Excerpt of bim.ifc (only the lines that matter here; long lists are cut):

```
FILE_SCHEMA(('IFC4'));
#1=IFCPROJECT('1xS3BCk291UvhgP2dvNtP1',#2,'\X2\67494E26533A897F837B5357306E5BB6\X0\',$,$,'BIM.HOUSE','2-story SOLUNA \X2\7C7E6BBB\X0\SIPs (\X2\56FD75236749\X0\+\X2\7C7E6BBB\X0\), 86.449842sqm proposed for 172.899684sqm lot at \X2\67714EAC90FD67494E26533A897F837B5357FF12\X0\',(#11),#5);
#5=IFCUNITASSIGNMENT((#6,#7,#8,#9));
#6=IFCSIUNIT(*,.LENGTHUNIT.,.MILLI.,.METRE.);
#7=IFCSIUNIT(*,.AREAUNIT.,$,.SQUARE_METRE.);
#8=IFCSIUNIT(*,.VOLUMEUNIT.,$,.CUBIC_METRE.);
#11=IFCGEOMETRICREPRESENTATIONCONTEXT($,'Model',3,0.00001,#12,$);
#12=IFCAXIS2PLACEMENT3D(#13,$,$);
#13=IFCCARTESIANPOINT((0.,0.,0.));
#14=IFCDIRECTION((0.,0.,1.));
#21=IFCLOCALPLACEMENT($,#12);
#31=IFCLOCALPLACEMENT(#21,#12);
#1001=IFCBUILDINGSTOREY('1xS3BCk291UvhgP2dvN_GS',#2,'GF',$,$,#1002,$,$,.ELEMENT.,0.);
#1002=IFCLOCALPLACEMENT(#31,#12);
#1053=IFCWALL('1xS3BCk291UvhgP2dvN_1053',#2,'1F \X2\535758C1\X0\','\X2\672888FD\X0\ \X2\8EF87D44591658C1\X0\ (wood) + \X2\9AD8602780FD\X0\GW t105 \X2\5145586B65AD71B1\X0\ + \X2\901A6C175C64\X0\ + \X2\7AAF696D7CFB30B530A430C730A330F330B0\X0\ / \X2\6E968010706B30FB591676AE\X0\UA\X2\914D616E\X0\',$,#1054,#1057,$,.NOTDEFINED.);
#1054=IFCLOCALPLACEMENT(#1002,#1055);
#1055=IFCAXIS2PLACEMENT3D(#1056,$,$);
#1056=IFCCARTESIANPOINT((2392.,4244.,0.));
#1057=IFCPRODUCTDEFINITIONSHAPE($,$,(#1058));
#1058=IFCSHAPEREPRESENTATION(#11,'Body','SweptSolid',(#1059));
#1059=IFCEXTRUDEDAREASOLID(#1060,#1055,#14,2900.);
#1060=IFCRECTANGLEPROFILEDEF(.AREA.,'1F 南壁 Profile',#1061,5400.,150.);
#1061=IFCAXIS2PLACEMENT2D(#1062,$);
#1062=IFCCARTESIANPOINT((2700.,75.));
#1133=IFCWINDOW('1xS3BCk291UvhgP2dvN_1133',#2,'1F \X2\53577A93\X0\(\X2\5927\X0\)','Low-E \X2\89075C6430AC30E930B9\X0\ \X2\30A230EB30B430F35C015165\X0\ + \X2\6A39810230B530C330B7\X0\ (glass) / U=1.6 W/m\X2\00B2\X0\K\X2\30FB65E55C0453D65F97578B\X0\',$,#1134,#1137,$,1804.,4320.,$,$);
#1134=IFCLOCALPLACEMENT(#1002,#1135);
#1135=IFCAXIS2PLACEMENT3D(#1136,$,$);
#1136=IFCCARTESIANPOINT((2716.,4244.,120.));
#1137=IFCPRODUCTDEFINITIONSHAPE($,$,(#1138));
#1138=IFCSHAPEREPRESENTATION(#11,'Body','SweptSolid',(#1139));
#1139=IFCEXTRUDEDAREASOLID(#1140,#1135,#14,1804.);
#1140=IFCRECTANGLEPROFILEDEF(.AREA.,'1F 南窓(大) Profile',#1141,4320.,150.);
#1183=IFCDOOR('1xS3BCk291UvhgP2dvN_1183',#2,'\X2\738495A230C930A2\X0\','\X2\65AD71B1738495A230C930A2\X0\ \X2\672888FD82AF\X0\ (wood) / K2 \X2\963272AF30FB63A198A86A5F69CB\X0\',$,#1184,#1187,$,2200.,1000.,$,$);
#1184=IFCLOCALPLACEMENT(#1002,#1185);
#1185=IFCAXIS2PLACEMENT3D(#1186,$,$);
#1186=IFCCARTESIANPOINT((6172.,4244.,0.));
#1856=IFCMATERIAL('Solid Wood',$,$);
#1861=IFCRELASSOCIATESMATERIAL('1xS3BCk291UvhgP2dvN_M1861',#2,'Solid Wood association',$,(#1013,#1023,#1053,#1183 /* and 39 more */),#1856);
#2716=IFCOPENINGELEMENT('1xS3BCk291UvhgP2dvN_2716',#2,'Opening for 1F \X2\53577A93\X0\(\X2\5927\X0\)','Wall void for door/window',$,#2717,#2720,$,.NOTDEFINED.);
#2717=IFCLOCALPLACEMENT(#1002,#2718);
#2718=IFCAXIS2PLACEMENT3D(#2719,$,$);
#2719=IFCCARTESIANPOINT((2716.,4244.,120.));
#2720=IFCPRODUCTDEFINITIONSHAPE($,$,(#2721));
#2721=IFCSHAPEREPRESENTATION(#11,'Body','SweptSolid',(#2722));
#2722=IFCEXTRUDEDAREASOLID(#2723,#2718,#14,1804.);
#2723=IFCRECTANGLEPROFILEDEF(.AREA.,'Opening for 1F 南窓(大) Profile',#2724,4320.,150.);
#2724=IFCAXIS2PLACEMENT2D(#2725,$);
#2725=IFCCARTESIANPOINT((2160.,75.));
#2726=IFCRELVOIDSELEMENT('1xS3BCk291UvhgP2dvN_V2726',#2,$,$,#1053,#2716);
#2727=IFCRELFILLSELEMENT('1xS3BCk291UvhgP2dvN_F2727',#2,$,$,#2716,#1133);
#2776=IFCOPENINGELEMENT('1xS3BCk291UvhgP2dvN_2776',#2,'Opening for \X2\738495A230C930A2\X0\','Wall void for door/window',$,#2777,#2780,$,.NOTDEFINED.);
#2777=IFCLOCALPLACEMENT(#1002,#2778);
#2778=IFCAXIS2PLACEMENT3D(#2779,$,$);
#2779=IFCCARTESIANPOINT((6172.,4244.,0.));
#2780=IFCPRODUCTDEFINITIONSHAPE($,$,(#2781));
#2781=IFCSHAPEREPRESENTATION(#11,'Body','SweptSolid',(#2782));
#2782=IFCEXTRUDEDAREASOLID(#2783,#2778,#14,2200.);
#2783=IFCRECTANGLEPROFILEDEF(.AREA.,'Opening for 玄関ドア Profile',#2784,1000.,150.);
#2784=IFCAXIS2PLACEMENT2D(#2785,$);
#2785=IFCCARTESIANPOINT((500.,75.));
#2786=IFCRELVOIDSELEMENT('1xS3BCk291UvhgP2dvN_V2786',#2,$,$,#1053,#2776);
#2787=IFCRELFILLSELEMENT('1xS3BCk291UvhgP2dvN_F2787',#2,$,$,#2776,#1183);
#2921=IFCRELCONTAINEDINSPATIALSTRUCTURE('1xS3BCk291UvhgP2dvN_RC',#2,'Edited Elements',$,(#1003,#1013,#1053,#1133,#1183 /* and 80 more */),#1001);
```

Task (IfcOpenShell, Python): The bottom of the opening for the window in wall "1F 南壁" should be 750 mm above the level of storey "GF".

```python
import numpy as np
import ifcopenshell
import ifcopenshell.api.geometry
import ifcopenshell.geom
import ifcopenshell.util.element
import ifcopenshell.util.placement
import ifcopenshell.util.shape
import ifcopenshell.util.unit

model = ifcopenshell.open("bim.ifc")
unit_scale = ifcopenshell.util.unit.calculate_unit_scale(model)

window = model.by_guid("1xS3BCk291UvhgP2dvN_1133")
opening = window.FillsVoids[0].RelatingOpeningElement
storey = ifcopenshell.util.element.get_container(window, ifc_class="IfcBuildingStorey")
level = ifcopenshell.util.placement.get_local_placement(storey.ObjectPlacement)[2, 3]

# The opening's origin need not be at the sill, so measure its lowest point.
shape = ifcopenshell.geom.create_shape(ifcopenshell.geom.settings(), opening)
bottom = ifcopenshell.util.shape.get_shape_bottom_elevation(shape, shape.geometry) / unit_scale
dz = level + 0.75 / unit_scale - bottom

shift = np.array([0.0, 0.0, dz])
# The window is not placed relative to its opening, so move both.
for product in (opening, window):
    matrix = ifcopenshell.util.placement.get_local_placement(product.ObjectPlacement)
    matrix[:3, 3] += shift
    ifcopenshell.api.geometry.edit_object_placement(model, product=product, matrix=matrix, is_si=False)

print(f"moved by {dz * unit_scale:+.3f} m")

model.write("bim_rev.ifc")
```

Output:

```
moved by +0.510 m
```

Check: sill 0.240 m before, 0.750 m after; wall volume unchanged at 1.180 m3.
